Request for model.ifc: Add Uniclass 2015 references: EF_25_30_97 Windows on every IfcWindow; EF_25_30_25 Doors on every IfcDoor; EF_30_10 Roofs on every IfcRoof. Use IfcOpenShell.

First a look at what the model holds.

```python
import ifcopenshell

model = ifcopenshell.open("model.ifc")
print(model.schema)
print("classifications:", [c.Name for c in model.by_type("IfcClassification")])
for ifc_class in ("IfcDoor", "IfcRoof", "IfcStair", "IfcWall", "IfcWindow"):
    print(ifc_class, len(model.by_type(ifc_class)))
```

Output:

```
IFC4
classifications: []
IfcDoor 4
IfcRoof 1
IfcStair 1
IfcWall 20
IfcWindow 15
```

```python
import ifcopenshell
import ifcopenshell.api.classification

model = ifcopenshell.open("model.ifc")

system = ifcopenshell.api.classification.add_classification(model, classification="Uniclass 2015")

codes = {
    "IfcWindow": ("EF_25_30_97", "Windows"),
    "IfcDoor": ("EF_25_30_25", "Doors"),
    "IfcRoof": ("EF_30_10", "Roofs"),
}
for ifc_class, (code, name) in codes.items():
    products = model.by_type(ifc_class)
    ifcopenshell.api.classification.add_reference(
        model, products=products, classification=system, identification=code, name=name
    )
    print(code, len(products))

model.write("model_edited.ifc")
```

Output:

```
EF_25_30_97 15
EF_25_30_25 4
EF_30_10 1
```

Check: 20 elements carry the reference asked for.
